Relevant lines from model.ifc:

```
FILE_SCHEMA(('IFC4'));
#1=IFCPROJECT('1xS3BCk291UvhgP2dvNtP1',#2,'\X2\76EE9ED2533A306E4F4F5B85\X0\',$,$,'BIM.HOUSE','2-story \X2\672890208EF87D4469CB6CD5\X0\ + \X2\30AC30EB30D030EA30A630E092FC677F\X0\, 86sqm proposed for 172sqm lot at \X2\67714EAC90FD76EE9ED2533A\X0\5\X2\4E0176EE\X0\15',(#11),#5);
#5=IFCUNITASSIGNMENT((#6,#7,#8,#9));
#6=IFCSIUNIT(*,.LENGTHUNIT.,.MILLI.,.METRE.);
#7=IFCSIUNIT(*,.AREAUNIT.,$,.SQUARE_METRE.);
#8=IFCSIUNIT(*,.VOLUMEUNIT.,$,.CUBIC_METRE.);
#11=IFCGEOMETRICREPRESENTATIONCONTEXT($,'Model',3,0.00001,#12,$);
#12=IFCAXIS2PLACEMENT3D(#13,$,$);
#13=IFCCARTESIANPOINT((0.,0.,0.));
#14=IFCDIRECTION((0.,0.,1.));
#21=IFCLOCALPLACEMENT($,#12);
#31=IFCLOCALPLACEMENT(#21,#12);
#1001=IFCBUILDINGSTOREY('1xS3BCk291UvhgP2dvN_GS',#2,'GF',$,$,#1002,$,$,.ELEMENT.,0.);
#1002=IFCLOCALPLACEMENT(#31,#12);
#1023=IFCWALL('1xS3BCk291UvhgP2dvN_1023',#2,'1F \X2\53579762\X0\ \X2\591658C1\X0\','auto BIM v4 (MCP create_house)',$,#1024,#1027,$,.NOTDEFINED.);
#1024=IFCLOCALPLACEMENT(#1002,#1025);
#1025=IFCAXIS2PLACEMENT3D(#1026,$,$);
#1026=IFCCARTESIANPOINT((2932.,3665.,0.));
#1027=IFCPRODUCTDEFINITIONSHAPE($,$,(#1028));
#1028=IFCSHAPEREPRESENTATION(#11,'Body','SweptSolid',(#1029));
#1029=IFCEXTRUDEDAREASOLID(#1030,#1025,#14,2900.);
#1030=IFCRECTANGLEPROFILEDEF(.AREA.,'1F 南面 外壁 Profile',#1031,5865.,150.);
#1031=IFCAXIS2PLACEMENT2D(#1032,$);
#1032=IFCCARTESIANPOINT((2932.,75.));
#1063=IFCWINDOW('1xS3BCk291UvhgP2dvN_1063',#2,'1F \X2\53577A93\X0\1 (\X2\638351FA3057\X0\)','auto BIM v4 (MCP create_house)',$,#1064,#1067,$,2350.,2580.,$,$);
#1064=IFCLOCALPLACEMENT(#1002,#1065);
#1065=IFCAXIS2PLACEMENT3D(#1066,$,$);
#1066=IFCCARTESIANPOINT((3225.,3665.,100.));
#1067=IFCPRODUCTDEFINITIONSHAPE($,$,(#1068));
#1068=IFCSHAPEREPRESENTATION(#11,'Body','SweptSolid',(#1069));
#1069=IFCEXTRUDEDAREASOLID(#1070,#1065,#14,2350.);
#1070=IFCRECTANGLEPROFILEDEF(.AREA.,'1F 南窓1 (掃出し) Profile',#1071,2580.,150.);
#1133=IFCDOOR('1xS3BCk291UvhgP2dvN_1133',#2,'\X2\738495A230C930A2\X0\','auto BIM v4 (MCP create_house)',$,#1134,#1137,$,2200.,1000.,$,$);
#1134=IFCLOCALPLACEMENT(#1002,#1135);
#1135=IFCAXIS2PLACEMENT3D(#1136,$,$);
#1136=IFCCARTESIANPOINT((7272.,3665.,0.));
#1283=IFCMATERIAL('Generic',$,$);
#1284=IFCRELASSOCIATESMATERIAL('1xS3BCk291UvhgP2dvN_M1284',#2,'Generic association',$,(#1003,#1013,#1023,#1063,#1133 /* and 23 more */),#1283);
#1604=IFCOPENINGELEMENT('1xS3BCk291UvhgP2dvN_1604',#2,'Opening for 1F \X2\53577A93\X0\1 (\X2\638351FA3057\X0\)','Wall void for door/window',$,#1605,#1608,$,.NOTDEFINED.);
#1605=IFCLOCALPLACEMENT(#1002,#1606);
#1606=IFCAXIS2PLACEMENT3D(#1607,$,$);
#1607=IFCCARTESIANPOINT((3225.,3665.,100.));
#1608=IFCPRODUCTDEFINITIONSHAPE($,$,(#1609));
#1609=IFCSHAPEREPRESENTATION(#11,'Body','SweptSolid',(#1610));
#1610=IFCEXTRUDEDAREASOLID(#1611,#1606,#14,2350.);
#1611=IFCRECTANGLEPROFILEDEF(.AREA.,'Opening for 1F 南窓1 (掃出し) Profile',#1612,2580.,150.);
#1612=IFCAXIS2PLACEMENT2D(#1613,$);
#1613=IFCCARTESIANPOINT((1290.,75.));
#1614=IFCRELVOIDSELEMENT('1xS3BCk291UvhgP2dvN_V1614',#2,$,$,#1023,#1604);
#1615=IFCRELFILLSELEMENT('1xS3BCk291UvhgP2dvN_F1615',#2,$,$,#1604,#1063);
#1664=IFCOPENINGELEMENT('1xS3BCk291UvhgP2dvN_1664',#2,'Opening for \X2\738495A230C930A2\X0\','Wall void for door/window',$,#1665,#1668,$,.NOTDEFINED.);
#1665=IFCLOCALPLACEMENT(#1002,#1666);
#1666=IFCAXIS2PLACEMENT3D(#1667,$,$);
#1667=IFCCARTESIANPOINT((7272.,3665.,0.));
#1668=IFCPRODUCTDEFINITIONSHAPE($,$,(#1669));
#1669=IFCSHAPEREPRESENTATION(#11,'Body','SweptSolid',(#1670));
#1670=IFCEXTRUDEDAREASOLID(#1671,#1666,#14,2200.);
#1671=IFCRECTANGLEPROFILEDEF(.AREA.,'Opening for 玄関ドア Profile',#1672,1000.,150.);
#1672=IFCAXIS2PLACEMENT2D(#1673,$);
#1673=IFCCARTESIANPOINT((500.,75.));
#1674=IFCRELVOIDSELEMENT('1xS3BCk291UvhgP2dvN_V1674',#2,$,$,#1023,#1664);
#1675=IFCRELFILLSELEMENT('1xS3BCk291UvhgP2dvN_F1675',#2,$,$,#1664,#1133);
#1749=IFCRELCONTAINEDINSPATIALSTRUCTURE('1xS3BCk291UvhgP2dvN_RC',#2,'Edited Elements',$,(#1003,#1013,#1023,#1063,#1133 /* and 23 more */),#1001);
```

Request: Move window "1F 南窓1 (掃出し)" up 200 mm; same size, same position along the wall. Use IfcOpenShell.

```python
import numpy as np
import ifcopenshell
import ifcopenshell.api.geometry
import ifcopenshell.util.placement
import ifcopenshell.util.unit

model = ifcopenshell.open("model.ifc")
unit_scale = ifcopenshell.util.unit.calculate_unit_scale(model)

window = model.by_id(1063)
opening = window.FillsVoids[0].RelatingOpeningElement
dz = 0.2 / unit_scale

shift = np.array([0.0, 0.0, dz])
# The window is not placed relative to its opening, so move both.
for product in (opening, window):
    matrix = ifcopenshell.util.placement.get_local_placement(product.ObjectPlacement)
    matrix[:3, 3] += shift
    ifcopenshell.api.geometry.edit_object_placement(model, product=product, matrix=matrix, is_si=False)

print(f"moved by {dz * unit_scale:+.3f} m")

model.write("model_edited.ifc")
```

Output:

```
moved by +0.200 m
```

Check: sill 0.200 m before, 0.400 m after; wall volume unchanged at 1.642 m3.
